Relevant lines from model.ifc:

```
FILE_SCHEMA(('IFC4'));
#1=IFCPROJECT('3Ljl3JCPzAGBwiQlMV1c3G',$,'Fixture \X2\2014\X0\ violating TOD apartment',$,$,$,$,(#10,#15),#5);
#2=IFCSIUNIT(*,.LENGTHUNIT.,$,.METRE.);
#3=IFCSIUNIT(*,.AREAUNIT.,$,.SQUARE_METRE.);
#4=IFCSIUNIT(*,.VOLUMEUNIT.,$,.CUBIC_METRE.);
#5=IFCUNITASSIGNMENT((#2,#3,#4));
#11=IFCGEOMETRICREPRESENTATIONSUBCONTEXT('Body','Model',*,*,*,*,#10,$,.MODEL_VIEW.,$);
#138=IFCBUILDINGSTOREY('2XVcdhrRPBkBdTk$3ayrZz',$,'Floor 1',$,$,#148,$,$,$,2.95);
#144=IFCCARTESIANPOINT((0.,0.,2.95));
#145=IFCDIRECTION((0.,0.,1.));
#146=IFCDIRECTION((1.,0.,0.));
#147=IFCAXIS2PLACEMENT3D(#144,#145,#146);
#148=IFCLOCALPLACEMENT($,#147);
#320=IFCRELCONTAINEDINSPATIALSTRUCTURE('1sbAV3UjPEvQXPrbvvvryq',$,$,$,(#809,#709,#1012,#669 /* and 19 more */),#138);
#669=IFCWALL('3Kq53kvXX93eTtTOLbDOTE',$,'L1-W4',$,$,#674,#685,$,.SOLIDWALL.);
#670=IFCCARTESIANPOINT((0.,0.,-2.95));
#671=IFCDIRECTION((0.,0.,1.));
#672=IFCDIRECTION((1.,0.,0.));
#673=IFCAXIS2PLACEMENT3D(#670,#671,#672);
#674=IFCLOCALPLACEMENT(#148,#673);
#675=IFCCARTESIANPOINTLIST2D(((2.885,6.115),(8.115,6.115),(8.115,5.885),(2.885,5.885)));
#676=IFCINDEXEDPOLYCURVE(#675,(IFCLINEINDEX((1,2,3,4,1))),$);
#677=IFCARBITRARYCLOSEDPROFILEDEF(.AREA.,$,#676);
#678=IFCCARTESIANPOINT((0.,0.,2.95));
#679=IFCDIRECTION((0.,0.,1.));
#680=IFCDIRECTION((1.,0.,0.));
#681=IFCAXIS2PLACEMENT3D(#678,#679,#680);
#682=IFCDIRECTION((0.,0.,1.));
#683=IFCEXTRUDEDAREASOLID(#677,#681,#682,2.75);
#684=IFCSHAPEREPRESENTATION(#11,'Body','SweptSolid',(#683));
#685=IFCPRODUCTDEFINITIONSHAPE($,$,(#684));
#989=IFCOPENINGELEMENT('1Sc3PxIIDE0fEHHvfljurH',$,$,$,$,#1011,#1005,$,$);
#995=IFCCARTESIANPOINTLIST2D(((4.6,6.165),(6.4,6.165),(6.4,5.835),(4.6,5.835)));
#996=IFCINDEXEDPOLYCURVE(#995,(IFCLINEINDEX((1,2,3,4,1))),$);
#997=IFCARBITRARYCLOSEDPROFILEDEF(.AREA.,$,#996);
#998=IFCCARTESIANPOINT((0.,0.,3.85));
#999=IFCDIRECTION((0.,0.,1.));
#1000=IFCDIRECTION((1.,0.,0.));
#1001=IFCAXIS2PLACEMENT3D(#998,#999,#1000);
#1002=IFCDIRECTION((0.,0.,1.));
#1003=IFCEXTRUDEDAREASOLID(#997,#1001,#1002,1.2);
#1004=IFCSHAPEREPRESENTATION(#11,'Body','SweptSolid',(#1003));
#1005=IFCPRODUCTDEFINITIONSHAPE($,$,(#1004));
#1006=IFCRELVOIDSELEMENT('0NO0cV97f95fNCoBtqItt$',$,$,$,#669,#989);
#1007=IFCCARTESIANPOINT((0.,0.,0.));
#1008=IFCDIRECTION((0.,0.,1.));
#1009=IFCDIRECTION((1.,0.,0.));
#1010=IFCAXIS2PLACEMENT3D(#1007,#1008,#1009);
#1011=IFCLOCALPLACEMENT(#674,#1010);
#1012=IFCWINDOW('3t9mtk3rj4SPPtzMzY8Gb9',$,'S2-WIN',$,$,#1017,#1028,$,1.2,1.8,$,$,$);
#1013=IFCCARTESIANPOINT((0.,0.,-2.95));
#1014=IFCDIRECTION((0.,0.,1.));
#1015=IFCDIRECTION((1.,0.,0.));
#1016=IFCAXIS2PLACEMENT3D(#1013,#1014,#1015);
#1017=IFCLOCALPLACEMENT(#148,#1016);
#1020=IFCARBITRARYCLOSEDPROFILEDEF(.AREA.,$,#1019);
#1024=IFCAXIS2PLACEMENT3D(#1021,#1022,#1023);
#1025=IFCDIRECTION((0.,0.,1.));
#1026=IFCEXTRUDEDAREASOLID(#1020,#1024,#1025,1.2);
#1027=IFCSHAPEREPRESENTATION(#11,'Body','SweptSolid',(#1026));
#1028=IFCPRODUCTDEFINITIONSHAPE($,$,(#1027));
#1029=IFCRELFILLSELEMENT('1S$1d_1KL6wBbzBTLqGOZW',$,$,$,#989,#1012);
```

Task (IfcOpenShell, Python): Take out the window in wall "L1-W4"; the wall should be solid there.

```python
import ifcopenshell
import ifcopenshell.api.feature
import ifcopenshell.api.root
import ifcopenshell.geom
import ifcopenshell.util.shape

model = ifcopenshell.open("model.ifc")
settings = ifcopenshell.geom.settings()


def volume(element):
    """Net volume in cubic metres, openings subtracted."""
    shape = ifcopenshell.geom.create_shape(settings, element)
    return ifcopenshell.util.shape.get_volume(shape.geometry)


window = model.by_id(1012)
opening = window.FillsVoids[0].RelatingOpeningElement
wall = opening.VoidsElements[0].RelatingBuildingElement
before = volume(wall)

ifcopenshell.api.root.remove_product(model, product=window)
ifcopenshell.api.feature.remove_feature(model, feature=opening)

after = volume(wall)

print(f"wall volume {before:.3f} -> {after:.3f} m3")

model.write("model_v2.ifc")
```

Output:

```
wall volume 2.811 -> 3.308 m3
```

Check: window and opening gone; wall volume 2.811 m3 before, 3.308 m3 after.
